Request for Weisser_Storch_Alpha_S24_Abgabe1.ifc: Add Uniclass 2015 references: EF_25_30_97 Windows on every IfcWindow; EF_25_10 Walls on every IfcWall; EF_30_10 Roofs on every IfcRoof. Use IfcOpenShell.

First a look at what the model holds.

```python
import ifcopenshell

model = ifcopenshell.open("Weisser_Storch_Alpha_S24_Abgabe1.ifc")
print(model.schema)
print("classifications:", [c.Name for c in model.by_type("IfcClassification")])
for ifc_class in ("IfcDoor", "IfcRoof", "IfcStair", "IfcWall", "IfcWindow"):
    print(ifc_class, len(model.by_type(ifc_class)))
```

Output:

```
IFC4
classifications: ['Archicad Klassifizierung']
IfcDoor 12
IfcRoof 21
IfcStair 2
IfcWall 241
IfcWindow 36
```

```python
import ifcopenshell
import ifcopenshell.api.classification

model = ifcopenshell.open("Weisser_Storch_Alpha_S24_Abgabe1.ifc")

system = ifcopenshell.api.classification.add_classification(model, classification="Uniclass 2015")

codes = {
    "IfcWindow": ("EF_25_30_97", "Windows"),
    "IfcWall": ("EF_25_10", "Walls"),
    "IfcRoof": ("EF_30_10", "Roofs"),
}
for ifc_class, (code, name) in codes.items():
    products = model.by_type(ifc_class)
    ifcopenshell.api.classification.add_reference(
        model, products=products, classification=system, identification=code, name=name
    )
    print(code, len(products))

model.write("Weisser_Storch_Alpha_S24_Abgabe1_v2.ifc")
```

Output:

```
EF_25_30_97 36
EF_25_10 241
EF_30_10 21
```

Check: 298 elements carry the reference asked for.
